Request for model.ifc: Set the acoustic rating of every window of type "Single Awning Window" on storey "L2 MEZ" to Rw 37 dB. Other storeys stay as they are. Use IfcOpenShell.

First a look at what the model holds.

```python
import ifcopenshell
import ifcopenshell.util.element

model = ifcopenshell.open("model.ifc")
print(model.schema)
storey = next(s for s in model.by_type("IfcBuildingStorey") if s.Name == "L2 MEZ")
windows = [e for e in ifcopenshell.util.element.get_decomposition(storey) if e.is_a("IfcWindow")]
seen = {}
for e in windows:
    element_type = ifcopenshell.util.element.get_type(e)
    key = (element_type.Name if element_type != e and element_type else None, ifcopenshell.util.element.get_pset(e, "Pset_WindowCommon", "AcousticRating"))
    seen[key] = seen.get(key, 0) + 1
for (name, value), count in sorted(seen.items(), key=str):
    print(count, "x", name, "|", value)
```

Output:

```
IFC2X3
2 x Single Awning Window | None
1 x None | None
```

```python
import ifcopenshell
import ifcopenshell.api.pset
import ifcopenshell.util.element

model = ifcopenshell.open("model.ifc")

storey = next(s for s in model.by_type("IfcBuildingStorey") if s.Name == "L2 MEZ")
windows = [e for e in ifcopenshell.util.element.get_decomposition(storey) if e.is_a("IfcWindow")]

count = 0
for e in windows:
    element_type = ifcopenshell.util.element.get_type(e)
    if element_type in (None, e) or element_type.Name != "Single Awning Window":
        continue
    # add_pset returns the element's existing set when there is one.
    pset = ifcopenshell.api.pset.add_pset(model, product=e, name="Pset_WindowCommon")
    ifcopenshell.api.pset.edit_pset(model, pset=pset, properties={"AcousticRating": "Rw 37 dB"})
    count += 1

print(count, "windows updated")

model.write("model-out.ifc")
```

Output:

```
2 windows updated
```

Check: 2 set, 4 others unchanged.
